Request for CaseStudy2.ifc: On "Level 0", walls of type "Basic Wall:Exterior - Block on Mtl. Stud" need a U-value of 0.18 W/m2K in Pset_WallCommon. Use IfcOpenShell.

First a look at what the model holds.

```python
import ifcopenshell
import ifcopenshell.util.element

model = ifcopenshell.open("CaseStudy2.ifc")
print(model.schema)
storey = next(s for s in model.by_type("IfcBuildingStorey") if s.Name == "Level 0")
walls = [e for e in ifcopenshell.util.element.get_decomposition(storey) if e.is_a("IfcWall")]
seen = {}
for e in walls:
    element_type = ifcopenshell.util.element.get_type(e)
    key = (element_type.Name if element_type != e and element_type else None, ifcopenshell.util.element.get_pset(e, "Pset_WallCommon", "ThermalTransmittance"))
    seen[key] = seen.get(key, 0) + 1
for (name, value), count in sorted(seen.items(), key=str):
    print(count, "x", name, "|", value)
```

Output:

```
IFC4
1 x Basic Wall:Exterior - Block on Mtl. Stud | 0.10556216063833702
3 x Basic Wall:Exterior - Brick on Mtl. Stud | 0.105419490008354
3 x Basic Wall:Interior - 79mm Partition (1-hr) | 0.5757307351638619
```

```python
import ifcopenshell
import ifcopenshell.api.pset
import ifcopenshell.util.element

model = ifcopenshell.open("CaseStudy2.ifc")

storey = next(s for s in model.by_type("IfcBuildingStorey") if s.Name == "Level 0")
walls = [e for e in ifcopenshell.util.element.get_decomposition(storey) if e.is_a("IfcWall")]

count = 0
for e in walls:
    element_type = ifcopenshell.util.element.get_type(e)
    if element_type in (None, e) or element_type.Name != "Basic Wall:Exterior - Block on Mtl. Stud":
        continue
    # add_pset returns the element's existing set when there is one.
    pset = ifcopenshell.api.pset.add_pset(model, product=e, name="Pset_WallCommon")
    ifcopenshell.api.pset.edit_pset(model, pset=pset, properties={"ThermalTransmittance": 0.18})
    count += 1

print(count, "walls updated")

model.write("CaseStudy2_edited.ifc")
```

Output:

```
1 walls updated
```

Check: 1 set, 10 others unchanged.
